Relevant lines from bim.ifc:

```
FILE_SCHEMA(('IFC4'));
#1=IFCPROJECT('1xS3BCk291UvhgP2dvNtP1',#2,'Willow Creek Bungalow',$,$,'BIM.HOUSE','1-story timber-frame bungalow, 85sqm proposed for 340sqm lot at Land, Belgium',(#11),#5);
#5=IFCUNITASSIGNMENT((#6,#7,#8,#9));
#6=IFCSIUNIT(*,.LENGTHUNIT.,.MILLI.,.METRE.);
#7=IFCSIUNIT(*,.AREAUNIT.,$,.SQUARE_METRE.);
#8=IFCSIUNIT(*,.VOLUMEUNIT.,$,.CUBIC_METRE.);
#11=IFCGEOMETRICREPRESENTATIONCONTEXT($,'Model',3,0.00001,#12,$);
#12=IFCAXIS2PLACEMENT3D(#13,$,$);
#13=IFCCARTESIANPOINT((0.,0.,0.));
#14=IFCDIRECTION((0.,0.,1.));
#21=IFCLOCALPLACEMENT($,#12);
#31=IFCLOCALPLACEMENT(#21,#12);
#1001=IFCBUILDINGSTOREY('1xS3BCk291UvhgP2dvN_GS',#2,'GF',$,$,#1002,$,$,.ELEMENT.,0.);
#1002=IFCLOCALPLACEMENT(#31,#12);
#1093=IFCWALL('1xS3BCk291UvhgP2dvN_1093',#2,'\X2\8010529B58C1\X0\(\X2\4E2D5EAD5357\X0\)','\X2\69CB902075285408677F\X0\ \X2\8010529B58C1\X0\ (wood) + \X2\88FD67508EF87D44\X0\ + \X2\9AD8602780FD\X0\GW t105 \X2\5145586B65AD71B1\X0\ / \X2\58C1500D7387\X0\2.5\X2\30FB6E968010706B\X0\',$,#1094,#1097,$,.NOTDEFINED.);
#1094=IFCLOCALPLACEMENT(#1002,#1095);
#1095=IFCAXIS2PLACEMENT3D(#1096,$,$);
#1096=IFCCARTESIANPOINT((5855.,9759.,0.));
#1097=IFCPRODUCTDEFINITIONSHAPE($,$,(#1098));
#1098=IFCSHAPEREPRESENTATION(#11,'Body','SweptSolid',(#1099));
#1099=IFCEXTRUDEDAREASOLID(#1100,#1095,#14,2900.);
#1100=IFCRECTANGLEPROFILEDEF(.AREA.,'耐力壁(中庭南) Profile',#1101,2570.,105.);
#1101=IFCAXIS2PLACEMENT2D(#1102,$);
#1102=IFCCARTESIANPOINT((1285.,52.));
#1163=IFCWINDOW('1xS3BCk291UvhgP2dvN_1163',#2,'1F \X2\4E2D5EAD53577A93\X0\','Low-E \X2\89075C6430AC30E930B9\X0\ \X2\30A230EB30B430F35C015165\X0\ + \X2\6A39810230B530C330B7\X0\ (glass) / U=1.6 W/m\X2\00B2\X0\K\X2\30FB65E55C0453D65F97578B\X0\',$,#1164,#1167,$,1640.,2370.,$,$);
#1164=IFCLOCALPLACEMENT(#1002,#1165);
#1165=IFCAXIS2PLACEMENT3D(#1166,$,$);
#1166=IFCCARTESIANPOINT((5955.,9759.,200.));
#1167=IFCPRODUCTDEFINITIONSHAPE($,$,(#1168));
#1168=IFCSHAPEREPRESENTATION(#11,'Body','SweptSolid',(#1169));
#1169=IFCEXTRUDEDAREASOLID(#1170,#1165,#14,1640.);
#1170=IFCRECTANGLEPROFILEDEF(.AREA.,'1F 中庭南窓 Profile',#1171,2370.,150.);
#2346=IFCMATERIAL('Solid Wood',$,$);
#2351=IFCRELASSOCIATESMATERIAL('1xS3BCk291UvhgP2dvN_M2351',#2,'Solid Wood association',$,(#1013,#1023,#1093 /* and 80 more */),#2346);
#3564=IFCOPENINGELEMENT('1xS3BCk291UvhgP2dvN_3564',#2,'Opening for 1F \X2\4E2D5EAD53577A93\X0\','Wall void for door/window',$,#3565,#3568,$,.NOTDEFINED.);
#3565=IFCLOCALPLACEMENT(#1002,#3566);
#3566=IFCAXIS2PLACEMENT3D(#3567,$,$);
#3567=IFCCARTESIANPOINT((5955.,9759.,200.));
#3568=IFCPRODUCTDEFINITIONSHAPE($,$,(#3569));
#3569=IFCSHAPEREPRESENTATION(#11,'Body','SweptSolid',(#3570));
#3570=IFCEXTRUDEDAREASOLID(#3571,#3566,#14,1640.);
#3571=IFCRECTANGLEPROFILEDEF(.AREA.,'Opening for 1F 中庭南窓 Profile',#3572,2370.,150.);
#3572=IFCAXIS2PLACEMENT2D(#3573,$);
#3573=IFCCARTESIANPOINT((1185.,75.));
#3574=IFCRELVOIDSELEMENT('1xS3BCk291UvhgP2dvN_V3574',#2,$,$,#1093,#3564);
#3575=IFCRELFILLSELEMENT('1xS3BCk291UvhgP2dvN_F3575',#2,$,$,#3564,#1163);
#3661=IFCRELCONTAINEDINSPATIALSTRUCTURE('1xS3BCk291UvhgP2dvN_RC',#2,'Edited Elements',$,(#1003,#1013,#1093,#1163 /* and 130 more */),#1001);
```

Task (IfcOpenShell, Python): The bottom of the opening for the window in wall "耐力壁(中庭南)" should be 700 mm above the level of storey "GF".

```python
import numpy as np
import ifcopenshell
import ifcopenshell.api.geometry
import ifcopenshell.geom
import ifcopenshell.util.element
import ifcopenshell.util.placement
import ifcopenshell.util.shape
import ifcopenshell.util.unit

model = ifcopenshell.open("bim.ifc")
unit_scale = ifcopenshell.util.unit.calculate_unit_scale(model)

window = model.by_guid("1xS3BCk291UvhgP2dvN_1163")
opening = window.FillsVoids[0].RelatingOpeningElement
storey = ifcopenshell.util.element.get_container(window, ifc_class="IfcBuildingStorey")
level = ifcopenshell.util.placement.get_local_placement(storey.ObjectPlacement)[2, 3]

# The opening's origin need not be at the sill, so measure its lowest point.
shape = ifcopenshell.geom.create_shape(ifcopenshell.geom.settings(), opening)
bottom = ifcopenshell.util.shape.get_shape_bottom_elevation(shape, shape.geometry) / unit_scale
dz = level + 0.7 / unit_scale - bottom

shift = np.array([0.0, 0.0, dz])
# The window is not placed relative to its opening, so move both.
for product in (opening, window):
    matrix = ifcopenshell.util.placement.get_local_placement(product.ObjectPlacement)
    matrix[:3, 3] += shift
    ifcopenshell.api.geometry.edit_object_placement(model, product=product, matrix=matrix, is_si=False)

print(f"moved by {dz * unit_scale:+.3f} m")

model.write("bim_v2.ifc")
```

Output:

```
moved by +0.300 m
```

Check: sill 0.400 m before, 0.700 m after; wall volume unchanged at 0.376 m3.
